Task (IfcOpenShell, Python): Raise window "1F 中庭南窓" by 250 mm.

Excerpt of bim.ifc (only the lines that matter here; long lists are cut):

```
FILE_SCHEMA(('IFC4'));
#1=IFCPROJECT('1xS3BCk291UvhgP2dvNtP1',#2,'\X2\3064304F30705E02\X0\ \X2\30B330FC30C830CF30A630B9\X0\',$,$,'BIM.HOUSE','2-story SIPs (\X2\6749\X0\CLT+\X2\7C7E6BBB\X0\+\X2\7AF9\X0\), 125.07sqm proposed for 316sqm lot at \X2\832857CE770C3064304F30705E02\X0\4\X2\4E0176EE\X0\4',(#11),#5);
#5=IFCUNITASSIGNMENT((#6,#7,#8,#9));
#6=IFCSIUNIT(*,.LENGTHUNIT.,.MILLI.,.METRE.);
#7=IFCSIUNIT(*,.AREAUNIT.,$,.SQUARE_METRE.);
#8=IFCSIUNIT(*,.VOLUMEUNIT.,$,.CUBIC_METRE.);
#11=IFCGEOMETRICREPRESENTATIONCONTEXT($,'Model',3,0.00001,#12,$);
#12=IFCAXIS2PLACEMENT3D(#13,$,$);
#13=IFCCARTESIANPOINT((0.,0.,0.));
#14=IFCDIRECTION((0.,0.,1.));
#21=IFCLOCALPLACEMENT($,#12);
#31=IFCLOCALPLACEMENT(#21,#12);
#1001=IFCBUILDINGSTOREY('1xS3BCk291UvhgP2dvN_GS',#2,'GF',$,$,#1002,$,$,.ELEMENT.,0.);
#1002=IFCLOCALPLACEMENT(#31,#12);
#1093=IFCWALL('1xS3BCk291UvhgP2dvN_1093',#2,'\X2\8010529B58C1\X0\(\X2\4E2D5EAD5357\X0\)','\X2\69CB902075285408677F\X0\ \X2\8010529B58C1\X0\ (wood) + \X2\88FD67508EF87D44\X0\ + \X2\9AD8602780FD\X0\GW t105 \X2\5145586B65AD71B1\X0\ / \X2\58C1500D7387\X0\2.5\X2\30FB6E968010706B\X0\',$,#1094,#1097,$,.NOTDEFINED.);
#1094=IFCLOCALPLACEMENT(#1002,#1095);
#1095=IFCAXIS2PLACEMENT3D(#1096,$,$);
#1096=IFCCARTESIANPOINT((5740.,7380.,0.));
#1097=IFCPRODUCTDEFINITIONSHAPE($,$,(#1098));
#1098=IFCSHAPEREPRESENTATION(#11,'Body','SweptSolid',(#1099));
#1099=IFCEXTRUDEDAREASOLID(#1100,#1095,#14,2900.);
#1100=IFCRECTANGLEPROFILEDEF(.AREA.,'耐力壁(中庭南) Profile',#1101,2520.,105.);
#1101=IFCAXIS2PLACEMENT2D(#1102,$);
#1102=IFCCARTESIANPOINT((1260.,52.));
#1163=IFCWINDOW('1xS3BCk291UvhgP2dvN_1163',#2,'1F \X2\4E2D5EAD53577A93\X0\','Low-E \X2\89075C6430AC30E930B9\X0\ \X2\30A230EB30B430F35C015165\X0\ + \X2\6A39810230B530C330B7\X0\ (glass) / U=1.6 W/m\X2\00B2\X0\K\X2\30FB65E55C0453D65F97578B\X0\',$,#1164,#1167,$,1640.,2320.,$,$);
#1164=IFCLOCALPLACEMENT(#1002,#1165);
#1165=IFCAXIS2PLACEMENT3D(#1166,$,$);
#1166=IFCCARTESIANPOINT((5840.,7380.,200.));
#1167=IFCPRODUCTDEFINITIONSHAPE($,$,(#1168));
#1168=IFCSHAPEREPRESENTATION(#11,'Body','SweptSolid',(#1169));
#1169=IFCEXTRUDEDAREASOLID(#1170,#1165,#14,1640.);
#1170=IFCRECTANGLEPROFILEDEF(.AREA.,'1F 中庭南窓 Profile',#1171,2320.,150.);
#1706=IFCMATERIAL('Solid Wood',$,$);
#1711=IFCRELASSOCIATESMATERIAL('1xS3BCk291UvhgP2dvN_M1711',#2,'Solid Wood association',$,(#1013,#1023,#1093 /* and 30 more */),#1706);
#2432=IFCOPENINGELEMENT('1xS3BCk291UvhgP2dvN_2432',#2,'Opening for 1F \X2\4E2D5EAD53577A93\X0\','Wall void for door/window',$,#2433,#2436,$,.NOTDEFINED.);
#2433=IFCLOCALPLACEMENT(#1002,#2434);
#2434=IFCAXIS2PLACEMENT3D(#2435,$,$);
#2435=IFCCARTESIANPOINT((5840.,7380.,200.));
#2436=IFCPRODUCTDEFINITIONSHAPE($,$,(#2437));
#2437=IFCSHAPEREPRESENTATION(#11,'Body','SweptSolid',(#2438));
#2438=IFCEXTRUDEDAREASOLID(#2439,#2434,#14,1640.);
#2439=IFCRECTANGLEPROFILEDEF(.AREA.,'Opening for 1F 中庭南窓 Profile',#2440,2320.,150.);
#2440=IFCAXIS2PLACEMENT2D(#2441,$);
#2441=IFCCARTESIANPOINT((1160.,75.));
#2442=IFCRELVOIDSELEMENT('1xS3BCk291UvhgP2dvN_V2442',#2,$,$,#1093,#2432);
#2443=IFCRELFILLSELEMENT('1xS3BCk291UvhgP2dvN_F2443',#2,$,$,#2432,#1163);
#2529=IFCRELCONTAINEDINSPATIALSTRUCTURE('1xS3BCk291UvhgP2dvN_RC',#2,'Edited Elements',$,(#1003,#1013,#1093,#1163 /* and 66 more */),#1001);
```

```python
import numpy as np
import ifcopenshell
import ifcopenshell.api.geometry
import ifcopenshell.util.placement
import ifcopenshell.util.unit

model = ifcopenshell.open("bim.ifc")
unit_scale = ifcopenshell.util.unit.calculate_unit_scale(model)

window = model.by_guid("1xS3BCk291UvhgP2dvN_1163")
opening = window.FillsVoids[0].RelatingOpeningElement
dz = 0.25 / unit_scale

shift = np.array([0.0, 0.0, dz])
# The window is not placed relative to its opening, so move both.
for product in (opening, window):
    matrix = ifcopenshell.util.placement.get_local_placement(product.ObjectPlacement)
    matrix[:3, 3] += shift
    ifcopenshell.api.geometry.edit_object_placement(model, product=product, matrix=matrix, is_si=False)

print(f"moved by {dz * unit_scale:+.3f} m")

model.write("bim_v2.ifc")
```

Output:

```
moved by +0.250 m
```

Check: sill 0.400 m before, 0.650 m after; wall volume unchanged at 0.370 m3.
